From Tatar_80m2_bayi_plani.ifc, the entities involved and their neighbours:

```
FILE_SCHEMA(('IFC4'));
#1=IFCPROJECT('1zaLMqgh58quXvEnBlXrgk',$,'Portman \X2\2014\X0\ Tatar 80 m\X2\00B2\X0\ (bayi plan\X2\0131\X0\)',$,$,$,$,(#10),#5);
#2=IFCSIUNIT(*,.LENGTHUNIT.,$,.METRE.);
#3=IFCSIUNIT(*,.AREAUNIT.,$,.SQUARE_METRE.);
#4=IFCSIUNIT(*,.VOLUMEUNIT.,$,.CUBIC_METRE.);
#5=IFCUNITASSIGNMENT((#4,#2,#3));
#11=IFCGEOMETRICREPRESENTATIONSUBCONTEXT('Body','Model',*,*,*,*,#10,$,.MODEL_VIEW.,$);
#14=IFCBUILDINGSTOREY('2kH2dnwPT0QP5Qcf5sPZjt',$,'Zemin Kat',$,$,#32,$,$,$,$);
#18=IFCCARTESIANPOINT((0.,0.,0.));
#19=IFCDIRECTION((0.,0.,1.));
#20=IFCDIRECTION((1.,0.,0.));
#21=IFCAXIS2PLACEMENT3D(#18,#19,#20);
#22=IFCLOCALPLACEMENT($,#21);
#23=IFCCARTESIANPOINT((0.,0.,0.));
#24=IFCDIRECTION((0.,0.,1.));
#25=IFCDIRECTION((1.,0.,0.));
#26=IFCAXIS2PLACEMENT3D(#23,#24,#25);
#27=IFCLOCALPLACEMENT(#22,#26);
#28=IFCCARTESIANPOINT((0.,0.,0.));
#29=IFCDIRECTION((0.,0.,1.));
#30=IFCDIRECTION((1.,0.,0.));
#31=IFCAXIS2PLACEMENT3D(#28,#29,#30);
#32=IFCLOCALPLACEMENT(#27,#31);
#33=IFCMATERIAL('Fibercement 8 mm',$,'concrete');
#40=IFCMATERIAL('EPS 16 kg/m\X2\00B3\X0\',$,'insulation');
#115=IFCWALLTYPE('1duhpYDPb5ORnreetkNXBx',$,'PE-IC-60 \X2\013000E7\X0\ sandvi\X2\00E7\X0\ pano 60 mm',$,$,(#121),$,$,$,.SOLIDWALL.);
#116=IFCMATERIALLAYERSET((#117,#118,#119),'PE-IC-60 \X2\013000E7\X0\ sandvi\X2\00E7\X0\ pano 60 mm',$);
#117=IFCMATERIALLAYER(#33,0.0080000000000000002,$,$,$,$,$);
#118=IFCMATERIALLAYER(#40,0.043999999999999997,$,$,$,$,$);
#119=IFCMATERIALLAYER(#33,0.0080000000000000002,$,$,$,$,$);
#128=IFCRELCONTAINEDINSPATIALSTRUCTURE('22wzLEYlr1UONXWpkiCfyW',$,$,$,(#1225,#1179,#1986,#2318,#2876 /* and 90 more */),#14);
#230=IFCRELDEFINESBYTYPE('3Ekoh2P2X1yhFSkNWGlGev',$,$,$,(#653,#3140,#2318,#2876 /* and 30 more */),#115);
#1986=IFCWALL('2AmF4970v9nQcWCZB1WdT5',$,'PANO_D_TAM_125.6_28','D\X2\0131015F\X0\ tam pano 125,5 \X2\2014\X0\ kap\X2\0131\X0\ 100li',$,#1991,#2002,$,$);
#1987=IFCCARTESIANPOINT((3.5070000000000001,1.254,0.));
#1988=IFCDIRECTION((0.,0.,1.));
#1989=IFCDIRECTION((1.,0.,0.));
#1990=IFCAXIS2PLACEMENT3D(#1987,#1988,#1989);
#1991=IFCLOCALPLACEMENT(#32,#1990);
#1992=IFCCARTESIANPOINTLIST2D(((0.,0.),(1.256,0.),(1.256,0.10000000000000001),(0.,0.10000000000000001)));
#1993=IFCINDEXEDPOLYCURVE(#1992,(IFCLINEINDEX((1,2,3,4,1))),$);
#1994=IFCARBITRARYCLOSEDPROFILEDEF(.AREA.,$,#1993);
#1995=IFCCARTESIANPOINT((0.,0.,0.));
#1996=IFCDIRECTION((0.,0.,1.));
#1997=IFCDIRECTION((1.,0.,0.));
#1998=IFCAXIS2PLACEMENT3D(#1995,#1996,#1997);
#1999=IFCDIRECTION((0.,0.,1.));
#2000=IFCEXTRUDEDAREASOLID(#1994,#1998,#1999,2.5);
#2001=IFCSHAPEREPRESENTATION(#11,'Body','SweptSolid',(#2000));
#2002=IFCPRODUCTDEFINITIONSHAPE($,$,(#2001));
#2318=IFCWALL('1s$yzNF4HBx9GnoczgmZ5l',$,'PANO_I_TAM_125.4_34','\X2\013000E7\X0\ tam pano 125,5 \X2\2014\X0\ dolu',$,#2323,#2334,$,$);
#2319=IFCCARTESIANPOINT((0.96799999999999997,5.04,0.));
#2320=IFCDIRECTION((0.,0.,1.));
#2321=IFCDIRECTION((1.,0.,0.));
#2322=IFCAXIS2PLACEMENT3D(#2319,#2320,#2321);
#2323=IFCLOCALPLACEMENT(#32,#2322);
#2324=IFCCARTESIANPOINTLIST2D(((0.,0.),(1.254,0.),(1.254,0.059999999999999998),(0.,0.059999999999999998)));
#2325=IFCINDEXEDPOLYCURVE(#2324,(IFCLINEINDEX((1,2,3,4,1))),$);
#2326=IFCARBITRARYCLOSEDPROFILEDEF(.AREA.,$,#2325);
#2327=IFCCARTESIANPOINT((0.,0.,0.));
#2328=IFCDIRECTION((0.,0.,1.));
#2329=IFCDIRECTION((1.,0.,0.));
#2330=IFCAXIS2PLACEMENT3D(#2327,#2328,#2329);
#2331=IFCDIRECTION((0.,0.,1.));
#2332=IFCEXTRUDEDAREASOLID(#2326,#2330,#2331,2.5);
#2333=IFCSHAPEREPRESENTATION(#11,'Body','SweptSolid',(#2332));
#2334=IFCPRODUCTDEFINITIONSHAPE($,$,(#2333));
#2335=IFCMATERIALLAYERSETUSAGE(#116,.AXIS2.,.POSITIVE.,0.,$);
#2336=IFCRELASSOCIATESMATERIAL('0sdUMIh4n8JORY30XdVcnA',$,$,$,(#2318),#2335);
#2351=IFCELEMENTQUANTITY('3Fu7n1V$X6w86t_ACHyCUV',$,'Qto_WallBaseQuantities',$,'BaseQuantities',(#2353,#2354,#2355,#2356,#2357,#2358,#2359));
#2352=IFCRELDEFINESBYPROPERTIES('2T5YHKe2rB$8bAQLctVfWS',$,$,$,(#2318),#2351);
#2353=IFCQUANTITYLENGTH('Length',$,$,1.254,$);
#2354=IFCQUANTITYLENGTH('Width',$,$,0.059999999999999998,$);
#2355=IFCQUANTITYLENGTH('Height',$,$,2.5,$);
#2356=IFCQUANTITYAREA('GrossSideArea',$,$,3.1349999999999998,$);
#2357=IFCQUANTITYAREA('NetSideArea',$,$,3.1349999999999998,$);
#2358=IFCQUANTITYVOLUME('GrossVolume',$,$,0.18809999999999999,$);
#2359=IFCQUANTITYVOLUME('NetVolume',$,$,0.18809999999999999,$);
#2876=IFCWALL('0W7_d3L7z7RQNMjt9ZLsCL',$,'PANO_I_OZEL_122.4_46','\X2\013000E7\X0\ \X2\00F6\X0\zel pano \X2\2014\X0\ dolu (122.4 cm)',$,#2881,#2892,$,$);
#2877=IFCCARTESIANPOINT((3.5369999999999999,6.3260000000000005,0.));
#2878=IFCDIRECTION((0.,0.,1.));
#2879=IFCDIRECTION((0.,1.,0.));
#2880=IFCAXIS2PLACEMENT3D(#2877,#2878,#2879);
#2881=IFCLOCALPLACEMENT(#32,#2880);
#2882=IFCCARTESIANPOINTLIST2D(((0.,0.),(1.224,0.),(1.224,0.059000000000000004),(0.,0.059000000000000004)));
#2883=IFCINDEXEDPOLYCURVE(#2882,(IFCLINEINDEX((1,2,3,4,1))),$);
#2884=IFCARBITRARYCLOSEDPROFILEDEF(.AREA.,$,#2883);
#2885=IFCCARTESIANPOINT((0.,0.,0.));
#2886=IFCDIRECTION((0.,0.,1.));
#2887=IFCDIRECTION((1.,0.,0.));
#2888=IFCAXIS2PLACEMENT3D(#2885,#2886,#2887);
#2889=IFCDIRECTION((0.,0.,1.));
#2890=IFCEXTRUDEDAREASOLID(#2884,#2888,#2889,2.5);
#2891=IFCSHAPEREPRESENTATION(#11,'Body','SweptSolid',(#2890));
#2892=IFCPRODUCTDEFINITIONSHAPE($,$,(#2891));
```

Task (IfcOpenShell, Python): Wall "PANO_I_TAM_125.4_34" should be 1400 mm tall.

```python
import ifcopenshell
import ifcopenshell.api.pset
import ifcopenshell.geom
import ifcopenshell.util.element
import ifcopenshell.util.representation
import ifcopenshell.util.shape
import ifcopenshell.util.unit

model = ifcopenshell.open("Tatar_80m2_bayi_plani.ifc")
unit_scale = ifcopenshell.util.unit.calculate_unit_scale(model)
area_scale = ifcopenshell.util.unit.calculate_unit_scale(model, "AREAUNIT")
volume_scale = ifcopenshell.util.unit.calculate_unit_scale(model, "VOLUMEUNIT")
settings = ifcopenshell.geom.settings()


def volume(element):
    """Net volume in cubic metres, openings subtracted."""
    shape = ifcopenshell.geom.create_shape(settings, element)
    return ifcopenshell.util.shape.get_volume(shape.geometry)


wall = model.by_guid("1s$yzNF4HBx9GnoczgmZ5l")
before = volume(wall)

body = ifcopenshell.util.representation.get_representation(wall, "Model", "Body")
solid = body.Items[0]
old_height = solid.Depth
solid.Depth = 1.4 / unit_scale
after = volume(wall)
thickness = 0.06  # wall thickness in metres

# Update the stored height, areas and volumes.
qto = model.by_id(ifcopenshell.util.element.get_pset(wall, "Qto_WallBaseQuantities", should_inherit=False)["id"])
ifcopenshell.api.pset.edit_qto(model, qto=qto, properties={
    "Height": solid.Depth,
    "GrossSideArea": ifcopenshell.util.element.get_pset(wall, "Qto_WallBaseQuantities", "GrossSideArea") * solid.Depth / old_height,
    "NetSideArea": after / thickness / area_scale,
    "GrossVolume": ifcopenshell.util.element.get_pset(wall, "Qto_WallBaseQuantities", "GrossVolume") * solid.Depth / old_height,
    "NetVolume": after / volume_scale,
})

print(f"height {old_height:g} -> {solid.Depth:g}, volume {before:.3f} -> {after:.3f} m3")

model.write("Tatar_80m2_bayi_plani_rev.ifc")
```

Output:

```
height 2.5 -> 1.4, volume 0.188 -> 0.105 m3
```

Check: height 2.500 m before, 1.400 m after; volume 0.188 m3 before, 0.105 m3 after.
